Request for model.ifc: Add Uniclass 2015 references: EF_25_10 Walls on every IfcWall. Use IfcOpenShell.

First a look at what the model holds.

```python
import ifcopenshell

model = ifcopenshell.open("model.ifc")
print(model.schema)
print("classifications:", [c.Name for c in model.by_type("IfcClassification")])
for ifc_class in ("IfcDoor", "IfcRoof", "IfcStair", "IfcWall", "IfcWindow"):
    print(ifc_class, len(model.by_type(ifc_class)))
```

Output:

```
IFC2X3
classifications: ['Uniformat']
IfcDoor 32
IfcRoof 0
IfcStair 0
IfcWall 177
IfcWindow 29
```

```python
import ifcopenshell
import ifcopenshell.api.classification

model = ifcopenshell.open("model.ifc")

# IFC2X3 requires Source and Edition and has no link from the project to the system.
system = model.create_entity("IfcClassification", Source="NBS", Edition="2015", Name="Uniclass 2015")

codes = {
    "IfcWall": ("EF_25_10", "Walls"),
}
for ifc_class, (code, name) in codes.items():
    products = model.by_type(ifc_class)
    ifcopenshell.api.classification.add_reference(
        model, products=products, classification=system, identification=code, name=name
    )
    print(code, len(products))

model.write("model-out.ifc")
```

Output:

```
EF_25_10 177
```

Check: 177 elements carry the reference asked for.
